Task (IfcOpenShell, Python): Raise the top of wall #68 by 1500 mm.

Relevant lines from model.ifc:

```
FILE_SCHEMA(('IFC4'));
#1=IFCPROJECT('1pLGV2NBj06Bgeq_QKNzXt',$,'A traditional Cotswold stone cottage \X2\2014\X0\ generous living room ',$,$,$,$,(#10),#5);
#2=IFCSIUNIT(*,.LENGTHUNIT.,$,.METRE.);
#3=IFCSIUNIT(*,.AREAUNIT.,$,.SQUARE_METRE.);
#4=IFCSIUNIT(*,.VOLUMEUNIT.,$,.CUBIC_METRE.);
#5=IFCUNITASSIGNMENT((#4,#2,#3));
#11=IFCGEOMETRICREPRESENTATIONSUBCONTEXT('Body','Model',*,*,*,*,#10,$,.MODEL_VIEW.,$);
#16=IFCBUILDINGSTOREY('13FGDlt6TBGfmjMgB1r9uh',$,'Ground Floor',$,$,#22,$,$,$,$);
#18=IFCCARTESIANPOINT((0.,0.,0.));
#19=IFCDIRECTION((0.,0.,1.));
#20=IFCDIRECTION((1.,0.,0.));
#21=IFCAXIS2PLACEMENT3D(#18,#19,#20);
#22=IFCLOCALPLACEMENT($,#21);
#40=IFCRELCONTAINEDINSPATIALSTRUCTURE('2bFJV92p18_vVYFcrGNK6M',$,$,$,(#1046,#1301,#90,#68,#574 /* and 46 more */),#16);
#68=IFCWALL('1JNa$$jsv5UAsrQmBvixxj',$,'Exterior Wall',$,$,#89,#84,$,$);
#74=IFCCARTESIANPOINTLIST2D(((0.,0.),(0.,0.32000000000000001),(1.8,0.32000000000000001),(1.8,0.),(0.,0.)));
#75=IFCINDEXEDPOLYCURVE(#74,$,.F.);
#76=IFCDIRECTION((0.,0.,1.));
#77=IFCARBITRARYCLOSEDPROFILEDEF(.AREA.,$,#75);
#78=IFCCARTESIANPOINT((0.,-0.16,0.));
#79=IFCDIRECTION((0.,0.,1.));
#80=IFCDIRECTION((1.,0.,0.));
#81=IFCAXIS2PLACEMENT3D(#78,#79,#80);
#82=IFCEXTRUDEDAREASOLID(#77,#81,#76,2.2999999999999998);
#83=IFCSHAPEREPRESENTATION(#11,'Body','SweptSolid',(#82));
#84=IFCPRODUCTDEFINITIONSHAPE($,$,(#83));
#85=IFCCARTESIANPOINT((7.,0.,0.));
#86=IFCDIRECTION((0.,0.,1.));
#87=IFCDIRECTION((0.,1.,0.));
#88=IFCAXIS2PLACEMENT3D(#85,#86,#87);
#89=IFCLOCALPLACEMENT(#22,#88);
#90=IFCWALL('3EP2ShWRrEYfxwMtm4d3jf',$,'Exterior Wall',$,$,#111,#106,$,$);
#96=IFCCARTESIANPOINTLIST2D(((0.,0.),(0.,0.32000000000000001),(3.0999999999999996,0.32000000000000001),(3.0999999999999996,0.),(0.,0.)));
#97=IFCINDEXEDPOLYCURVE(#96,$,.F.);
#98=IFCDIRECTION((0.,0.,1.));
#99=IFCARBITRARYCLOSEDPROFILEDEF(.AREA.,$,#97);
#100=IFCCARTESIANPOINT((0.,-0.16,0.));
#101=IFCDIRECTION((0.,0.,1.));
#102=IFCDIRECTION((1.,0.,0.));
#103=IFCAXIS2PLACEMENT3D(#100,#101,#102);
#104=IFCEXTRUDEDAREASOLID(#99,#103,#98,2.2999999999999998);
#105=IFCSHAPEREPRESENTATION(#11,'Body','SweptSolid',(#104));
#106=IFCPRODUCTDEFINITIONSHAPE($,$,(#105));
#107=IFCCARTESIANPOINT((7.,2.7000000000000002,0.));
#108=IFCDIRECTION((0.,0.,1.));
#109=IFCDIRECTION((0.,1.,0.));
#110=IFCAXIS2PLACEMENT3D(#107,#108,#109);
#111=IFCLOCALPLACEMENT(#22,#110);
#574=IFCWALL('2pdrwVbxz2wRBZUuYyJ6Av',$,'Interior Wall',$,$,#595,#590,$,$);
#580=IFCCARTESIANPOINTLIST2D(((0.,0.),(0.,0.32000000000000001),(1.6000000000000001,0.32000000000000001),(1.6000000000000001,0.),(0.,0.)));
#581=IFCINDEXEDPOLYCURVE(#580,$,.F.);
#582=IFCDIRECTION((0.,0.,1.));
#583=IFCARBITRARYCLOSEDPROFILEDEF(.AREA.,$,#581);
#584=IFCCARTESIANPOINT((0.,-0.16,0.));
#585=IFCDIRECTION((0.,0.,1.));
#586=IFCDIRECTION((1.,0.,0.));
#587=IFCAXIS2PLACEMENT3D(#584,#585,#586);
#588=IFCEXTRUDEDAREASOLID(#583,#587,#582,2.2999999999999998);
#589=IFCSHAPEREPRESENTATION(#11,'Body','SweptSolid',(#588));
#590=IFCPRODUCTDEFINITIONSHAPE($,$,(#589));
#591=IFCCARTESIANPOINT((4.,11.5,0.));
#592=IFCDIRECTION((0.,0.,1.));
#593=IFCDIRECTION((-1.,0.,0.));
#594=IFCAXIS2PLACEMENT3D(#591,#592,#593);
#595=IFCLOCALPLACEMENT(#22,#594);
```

```python
import ifcopenshell
import ifcopenshell.geom
import ifcopenshell.util.representation
import ifcopenshell.util.shape
import ifcopenshell.util.unit

model = ifcopenshell.open("model.ifc")
unit_scale = ifcopenshell.util.unit.calculate_unit_scale(model)
settings = ifcopenshell.geom.settings()


def volume(element):
    """Net volume in cubic metres, openings subtracted."""
    shape = ifcopenshell.geom.create_shape(settings, element)
    return ifcopenshell.util.shape.get_volume(shape.geometry)


wall = model.by_guid("1JNa$$jsv5UAsrQmBvixxj")
before = volume(wall)

body = ifcopenshell.util.representation.get_representation(wall, "Model", "Body")
solid = body.Items[0]
old_height = solid.Depth
solid.Depth += 1.5 / unit_scale
after = volume(wall)

print(f"height {old_height:g} -> {solid.Depth:g}, volume {before:.3f} -> {after:.3f} m3")

model.write("model_edited.ifc")
```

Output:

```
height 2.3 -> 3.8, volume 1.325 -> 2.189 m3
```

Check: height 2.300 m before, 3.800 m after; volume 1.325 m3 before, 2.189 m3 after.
